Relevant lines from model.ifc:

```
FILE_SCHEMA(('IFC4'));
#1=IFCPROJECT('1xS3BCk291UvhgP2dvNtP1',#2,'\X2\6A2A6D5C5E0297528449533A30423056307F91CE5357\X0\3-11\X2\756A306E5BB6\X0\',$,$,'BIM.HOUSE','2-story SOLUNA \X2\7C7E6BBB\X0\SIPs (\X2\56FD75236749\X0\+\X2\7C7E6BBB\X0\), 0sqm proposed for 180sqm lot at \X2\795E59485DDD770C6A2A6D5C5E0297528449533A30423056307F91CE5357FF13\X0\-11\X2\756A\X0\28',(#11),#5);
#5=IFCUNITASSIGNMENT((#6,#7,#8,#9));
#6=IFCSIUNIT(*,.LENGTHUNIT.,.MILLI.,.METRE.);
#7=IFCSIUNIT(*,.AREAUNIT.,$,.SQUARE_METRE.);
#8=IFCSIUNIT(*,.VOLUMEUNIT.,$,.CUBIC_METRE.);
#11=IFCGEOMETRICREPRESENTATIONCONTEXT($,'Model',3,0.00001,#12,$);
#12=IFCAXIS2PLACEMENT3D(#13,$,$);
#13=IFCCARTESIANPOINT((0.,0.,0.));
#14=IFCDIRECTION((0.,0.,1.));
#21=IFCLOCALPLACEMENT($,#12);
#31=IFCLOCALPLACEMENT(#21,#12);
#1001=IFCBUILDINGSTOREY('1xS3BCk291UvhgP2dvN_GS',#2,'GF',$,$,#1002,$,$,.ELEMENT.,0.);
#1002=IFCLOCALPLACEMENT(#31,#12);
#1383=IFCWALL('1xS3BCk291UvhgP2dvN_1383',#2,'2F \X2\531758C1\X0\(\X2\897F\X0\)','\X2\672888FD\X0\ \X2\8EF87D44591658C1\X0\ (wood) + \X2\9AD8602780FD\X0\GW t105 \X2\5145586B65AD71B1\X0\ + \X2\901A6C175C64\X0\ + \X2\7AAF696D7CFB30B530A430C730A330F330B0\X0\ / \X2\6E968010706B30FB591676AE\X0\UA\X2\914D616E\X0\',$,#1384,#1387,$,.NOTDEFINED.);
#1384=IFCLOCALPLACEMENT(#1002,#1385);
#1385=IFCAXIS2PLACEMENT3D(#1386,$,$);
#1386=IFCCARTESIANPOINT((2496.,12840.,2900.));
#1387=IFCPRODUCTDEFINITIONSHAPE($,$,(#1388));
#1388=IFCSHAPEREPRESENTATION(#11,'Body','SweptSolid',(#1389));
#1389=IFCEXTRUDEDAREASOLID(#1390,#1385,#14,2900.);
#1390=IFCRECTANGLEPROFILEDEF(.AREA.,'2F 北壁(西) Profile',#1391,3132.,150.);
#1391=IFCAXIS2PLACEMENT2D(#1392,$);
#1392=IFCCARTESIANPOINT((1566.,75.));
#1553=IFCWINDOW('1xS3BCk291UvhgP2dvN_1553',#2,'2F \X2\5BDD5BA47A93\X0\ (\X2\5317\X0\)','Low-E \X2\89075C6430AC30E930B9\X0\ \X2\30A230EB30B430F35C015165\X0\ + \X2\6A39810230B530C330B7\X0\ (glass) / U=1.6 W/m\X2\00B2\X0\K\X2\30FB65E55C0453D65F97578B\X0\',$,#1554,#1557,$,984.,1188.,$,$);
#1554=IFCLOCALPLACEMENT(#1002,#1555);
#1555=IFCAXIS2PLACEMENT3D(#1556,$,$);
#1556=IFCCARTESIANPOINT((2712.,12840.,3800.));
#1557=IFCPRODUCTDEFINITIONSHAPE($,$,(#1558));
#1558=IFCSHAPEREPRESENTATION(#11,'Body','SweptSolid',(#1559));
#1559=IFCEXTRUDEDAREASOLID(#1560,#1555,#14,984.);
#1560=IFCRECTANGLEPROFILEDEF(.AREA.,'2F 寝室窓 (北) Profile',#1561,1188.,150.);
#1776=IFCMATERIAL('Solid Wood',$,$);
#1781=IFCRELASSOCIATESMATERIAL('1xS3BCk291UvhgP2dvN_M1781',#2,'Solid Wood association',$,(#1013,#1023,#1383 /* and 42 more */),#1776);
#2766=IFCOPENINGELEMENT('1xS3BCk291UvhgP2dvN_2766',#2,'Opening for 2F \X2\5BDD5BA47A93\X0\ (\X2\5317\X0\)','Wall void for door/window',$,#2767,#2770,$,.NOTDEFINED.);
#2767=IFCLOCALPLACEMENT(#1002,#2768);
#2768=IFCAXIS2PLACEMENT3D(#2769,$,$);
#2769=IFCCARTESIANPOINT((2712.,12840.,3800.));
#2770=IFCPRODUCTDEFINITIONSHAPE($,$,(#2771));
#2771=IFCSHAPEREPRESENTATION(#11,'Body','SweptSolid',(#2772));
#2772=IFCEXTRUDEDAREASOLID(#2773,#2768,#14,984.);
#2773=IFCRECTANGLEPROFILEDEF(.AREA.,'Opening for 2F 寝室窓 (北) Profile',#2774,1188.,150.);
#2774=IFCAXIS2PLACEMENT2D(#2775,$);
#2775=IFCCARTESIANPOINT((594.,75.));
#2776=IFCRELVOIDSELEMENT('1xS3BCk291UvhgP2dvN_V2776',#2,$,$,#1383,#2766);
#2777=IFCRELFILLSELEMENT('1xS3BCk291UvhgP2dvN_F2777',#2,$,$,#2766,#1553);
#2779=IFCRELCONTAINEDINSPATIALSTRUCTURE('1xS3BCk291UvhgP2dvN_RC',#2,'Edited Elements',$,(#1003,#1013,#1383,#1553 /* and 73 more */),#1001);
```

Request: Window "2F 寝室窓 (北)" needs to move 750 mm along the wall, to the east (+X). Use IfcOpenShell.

```python
import ifcopenshell
import ifcopenshell.api.geometry
import ifcopenshell.util.placement
import ifcopenshell.util.unit

model = ifcopenshell.open("model.ifc")
unit_scale = ifcopenshell.util.unit.calculate_unit_scale(model)

window = model.by_guid("1xS3BCk291UvhgP2dvN_1553")
opening = window.FillsVoids[0].RelatingOpeningElement
wall = opening.VoidsElements[0].RelatingBuildingElement

wall_matrix = ifcopenshell.util.placement.get_local_placement(wall.ObjectPlacement)
shift = wall_matrix[:3, 0] * 0.75 / unit_scale
before = ifcopenshell.util.placement.get_local_placement(window.ObjectPlacement)[:3, 3].copy()

# The window is not placed relative to its opening, so move both.
for product in (opening, window):
    matrix = ifcopenshell.util.placement.get_local_placement(product.ObjectPlacement)
    matrix[:3, 3] += shift
    ifcopenshell.api.geometry.edit_object_placement(model, product=product, matrix=matrix, is_si=False)

after = ifcopenshell.util.placement.get_local_placement(window.ObjectPlacement)[:3, 3]
print("window moved by", (after - before).round(3) + 0.0)

model.write("model_rev.ifc")
```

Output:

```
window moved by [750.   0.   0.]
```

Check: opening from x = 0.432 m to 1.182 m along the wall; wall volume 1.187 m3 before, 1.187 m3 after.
